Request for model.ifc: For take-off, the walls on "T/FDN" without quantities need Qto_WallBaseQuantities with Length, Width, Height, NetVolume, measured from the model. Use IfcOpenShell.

First a look at what the model holds.

```python
import ifcopenshell
import ifcopenshell.util.element
import ifcopenshell.util.unit

model = ifcopenshell.open("model.ifc")
print(model.schema)
for unit_type in ("LENGTHUNIT", "AREAUNIT", "VOLUMEUNIT"):
    print(unit_type, ifcopenshell.util.unit.calculate_unit_scale(model, unit_type))
storey = next(s for s in model.by_type("IfcBuildingStorey") if s.Name == "T/FDN")
walls = [e for e in ifcopenshell.util.element.get_decomposition(storey) if e.is_a("IfcWall")]
for e in sorted(walls, key=lambda e: e.id()):
    print(e.id(), e.is_a(), e.Name, list(ifcopenshell.util.element.get_psets(e, qtos_only=True)), sep=" | ")
```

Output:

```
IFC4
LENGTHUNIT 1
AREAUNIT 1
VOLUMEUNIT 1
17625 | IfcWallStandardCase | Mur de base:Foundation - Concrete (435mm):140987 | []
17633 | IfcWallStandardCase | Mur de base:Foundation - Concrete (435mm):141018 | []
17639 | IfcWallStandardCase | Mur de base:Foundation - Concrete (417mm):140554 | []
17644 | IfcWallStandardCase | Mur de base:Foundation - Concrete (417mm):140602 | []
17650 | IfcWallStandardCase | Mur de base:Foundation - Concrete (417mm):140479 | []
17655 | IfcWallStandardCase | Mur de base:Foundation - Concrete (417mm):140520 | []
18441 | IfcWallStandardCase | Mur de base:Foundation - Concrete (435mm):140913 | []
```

```python
import ifcopenshell
import ifcopenshell.api.pset
import ifcopenshell.geom
import ifcopenshell.util.element
import ifcopenshell.util.shape
import ifcopenshell.util.unit

model = ifcopenshell.open("model.ifc")
unit_scale = ifcopenshell.util.unit.calculate_unit_scale(model)
volume_scale = ifcopenshell.util.unit.calculate_unit_scale(model, "VOLUMEUNIT")
settings = ifcopenshell.geom.settings()

storey = next(s for s in model.by_type("IfcBuildingStorey") if s.Name == "T/FDN")
walls = [e for e in ifcopenshell.util.element.get_decomposition(storey) if e.is_a("IfcWall")]

for e in sorted(walls, key=lambda e: e.id()):
    if ifcopenshell.util.element.get_psets(e, qtos_only=True, should_inherit=False):
        continue
    # Geometry comes back in metres, in the element's own axes.
    shape = ifcopenshell.geom.create_shape(settings, e)
    values = {
        "Length": ifcopenshell.util.shape.get_x(shape.geometry) / unit_scale,
        "Width": ifcopenshell.util.shape.get_y(shape.geometry) / unit_scale,
        "Height": ifcopenshell.util.shape.get_z(shape.geometry) / unit_scale,
        "NetVolume": ifcopenshell.util.shape.get_volume(shape.geometry) / volume_scale,
    }
    qto = ifcopenshell.api.pset.add_qto(model, product=e, name="Qto_WallBaseQuantities")
    ifcopenshell.api.pset.edit_qto(model, qto=qto, properties=values)
    print(e.id(), {k: round(v, 3) for k, v in values.items()})

model.write("model-out.ifc")
```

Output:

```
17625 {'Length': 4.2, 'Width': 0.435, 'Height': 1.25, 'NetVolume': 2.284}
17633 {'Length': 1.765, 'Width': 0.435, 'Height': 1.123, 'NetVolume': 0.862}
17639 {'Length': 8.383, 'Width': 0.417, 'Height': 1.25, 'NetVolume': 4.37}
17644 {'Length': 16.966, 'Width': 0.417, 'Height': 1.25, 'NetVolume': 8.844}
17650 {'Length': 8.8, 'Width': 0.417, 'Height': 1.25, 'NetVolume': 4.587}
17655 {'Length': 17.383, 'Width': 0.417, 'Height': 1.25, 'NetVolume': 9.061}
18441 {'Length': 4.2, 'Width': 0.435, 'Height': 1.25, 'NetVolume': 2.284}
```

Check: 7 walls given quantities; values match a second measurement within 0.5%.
